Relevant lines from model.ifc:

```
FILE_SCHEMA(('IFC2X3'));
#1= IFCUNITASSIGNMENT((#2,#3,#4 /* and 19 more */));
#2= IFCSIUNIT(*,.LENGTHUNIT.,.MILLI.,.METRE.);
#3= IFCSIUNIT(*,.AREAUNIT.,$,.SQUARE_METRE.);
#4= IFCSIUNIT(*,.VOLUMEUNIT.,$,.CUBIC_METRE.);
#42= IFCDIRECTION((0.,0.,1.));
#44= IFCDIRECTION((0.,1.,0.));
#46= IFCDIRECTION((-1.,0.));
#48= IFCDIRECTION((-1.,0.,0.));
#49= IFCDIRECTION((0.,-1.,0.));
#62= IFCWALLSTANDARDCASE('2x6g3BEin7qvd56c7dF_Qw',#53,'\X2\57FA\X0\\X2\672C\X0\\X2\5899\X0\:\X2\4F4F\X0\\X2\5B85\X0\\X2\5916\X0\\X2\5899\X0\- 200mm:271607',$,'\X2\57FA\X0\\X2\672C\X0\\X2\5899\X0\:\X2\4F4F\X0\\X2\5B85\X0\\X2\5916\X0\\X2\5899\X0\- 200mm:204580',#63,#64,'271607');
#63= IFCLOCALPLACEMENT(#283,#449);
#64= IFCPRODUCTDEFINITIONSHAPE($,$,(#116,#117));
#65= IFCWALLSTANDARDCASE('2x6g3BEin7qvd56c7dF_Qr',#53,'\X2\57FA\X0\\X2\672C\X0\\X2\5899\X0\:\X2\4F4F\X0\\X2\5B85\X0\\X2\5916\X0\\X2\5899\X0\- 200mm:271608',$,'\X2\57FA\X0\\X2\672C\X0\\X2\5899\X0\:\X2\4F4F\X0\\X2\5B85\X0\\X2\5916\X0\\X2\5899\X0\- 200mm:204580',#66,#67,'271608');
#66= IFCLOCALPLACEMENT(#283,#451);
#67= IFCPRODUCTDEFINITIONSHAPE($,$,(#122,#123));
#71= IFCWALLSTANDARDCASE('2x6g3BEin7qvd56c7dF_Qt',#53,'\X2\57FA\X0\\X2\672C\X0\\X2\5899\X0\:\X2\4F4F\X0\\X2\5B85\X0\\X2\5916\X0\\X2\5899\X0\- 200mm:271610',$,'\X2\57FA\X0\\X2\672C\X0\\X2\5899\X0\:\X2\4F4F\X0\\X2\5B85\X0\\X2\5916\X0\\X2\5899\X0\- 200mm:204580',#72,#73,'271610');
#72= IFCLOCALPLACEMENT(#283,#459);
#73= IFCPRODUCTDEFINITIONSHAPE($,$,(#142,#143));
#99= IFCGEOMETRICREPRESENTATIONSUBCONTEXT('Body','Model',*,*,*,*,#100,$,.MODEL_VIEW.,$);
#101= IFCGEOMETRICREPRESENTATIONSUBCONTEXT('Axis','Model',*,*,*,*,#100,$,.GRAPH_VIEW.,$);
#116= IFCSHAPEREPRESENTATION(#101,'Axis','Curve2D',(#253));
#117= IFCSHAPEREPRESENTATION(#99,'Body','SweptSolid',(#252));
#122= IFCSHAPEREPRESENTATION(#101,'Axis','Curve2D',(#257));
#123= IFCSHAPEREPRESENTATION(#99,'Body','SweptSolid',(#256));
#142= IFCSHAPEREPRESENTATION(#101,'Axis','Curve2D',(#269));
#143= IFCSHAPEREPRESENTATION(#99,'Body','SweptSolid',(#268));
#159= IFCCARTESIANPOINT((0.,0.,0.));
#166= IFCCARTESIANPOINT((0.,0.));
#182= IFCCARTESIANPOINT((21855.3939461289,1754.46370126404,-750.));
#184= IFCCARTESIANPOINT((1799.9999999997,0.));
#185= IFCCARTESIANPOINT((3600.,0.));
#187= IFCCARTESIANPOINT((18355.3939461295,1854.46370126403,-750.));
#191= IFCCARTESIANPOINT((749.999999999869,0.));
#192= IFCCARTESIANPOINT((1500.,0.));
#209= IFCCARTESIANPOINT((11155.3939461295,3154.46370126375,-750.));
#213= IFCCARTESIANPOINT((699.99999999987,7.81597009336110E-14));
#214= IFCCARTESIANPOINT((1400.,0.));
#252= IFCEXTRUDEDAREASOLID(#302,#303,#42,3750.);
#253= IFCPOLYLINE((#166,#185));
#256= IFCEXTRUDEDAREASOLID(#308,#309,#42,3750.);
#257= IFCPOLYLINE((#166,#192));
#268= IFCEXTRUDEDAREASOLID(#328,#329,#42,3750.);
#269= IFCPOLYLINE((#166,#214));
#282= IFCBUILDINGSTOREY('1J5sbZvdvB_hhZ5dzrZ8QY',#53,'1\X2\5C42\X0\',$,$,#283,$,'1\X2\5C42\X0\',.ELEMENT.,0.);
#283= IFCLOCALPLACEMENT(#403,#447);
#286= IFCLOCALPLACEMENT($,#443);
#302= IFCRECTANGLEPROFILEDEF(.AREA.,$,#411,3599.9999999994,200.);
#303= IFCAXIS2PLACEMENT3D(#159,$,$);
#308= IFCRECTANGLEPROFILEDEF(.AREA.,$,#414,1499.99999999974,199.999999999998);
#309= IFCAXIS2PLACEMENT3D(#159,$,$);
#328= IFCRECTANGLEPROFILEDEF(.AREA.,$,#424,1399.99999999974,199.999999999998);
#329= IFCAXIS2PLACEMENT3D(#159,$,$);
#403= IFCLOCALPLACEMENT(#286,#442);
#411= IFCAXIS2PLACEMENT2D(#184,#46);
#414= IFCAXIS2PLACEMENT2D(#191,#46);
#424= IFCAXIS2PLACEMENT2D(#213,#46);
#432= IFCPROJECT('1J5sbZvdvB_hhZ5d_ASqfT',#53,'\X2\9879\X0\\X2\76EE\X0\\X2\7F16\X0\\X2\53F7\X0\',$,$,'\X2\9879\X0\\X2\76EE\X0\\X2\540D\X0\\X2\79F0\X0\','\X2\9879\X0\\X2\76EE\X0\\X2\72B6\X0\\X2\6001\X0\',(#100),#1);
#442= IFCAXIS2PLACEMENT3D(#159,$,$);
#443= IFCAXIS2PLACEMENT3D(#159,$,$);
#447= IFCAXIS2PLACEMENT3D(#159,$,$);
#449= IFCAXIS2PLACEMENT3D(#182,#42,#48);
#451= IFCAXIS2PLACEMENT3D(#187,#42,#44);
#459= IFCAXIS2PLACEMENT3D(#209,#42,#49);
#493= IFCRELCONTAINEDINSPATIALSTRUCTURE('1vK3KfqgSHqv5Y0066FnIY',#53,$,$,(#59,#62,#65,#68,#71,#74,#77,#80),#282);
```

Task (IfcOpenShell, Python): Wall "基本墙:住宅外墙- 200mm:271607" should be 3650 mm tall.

```python
import ifcopenshell
import ifcopenshell.geom
import ifcopenshell.util.representation
import ifcopenshell.util.shape
import ifcopenshell.util.unit

model = ifcopenshell.open("model.ifc")
unit_scale = ifcopenshell.util.unit.calculate_unit_scale(model)
settings = ifcopenshell.geom.settings()


def volume(element):
    """Net volume in cubic metres, openings subtracted."""
    shape = ifcopenshell.geom.create_shape(settings, element)
    return ifcopenshell.util.shape.get_volume(shape.geometry)


wall = model.by_id(62)
before = volume(wall)

body = ifcopenshell.util.representation.get_representation(wall, "Model", "Body")
solid = body.Items[0]
old_height = solid.Depth
solid.Depth = 3.65 / unit_scale
after = volume(wall)

print(f"height {old_height:g} -> {solid.Depth:g}, volume {before:.3f} -> {after:.3f} m3")

model.write("model-out.ifc")
```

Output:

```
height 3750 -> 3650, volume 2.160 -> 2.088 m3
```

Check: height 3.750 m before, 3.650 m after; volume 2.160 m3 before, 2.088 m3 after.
